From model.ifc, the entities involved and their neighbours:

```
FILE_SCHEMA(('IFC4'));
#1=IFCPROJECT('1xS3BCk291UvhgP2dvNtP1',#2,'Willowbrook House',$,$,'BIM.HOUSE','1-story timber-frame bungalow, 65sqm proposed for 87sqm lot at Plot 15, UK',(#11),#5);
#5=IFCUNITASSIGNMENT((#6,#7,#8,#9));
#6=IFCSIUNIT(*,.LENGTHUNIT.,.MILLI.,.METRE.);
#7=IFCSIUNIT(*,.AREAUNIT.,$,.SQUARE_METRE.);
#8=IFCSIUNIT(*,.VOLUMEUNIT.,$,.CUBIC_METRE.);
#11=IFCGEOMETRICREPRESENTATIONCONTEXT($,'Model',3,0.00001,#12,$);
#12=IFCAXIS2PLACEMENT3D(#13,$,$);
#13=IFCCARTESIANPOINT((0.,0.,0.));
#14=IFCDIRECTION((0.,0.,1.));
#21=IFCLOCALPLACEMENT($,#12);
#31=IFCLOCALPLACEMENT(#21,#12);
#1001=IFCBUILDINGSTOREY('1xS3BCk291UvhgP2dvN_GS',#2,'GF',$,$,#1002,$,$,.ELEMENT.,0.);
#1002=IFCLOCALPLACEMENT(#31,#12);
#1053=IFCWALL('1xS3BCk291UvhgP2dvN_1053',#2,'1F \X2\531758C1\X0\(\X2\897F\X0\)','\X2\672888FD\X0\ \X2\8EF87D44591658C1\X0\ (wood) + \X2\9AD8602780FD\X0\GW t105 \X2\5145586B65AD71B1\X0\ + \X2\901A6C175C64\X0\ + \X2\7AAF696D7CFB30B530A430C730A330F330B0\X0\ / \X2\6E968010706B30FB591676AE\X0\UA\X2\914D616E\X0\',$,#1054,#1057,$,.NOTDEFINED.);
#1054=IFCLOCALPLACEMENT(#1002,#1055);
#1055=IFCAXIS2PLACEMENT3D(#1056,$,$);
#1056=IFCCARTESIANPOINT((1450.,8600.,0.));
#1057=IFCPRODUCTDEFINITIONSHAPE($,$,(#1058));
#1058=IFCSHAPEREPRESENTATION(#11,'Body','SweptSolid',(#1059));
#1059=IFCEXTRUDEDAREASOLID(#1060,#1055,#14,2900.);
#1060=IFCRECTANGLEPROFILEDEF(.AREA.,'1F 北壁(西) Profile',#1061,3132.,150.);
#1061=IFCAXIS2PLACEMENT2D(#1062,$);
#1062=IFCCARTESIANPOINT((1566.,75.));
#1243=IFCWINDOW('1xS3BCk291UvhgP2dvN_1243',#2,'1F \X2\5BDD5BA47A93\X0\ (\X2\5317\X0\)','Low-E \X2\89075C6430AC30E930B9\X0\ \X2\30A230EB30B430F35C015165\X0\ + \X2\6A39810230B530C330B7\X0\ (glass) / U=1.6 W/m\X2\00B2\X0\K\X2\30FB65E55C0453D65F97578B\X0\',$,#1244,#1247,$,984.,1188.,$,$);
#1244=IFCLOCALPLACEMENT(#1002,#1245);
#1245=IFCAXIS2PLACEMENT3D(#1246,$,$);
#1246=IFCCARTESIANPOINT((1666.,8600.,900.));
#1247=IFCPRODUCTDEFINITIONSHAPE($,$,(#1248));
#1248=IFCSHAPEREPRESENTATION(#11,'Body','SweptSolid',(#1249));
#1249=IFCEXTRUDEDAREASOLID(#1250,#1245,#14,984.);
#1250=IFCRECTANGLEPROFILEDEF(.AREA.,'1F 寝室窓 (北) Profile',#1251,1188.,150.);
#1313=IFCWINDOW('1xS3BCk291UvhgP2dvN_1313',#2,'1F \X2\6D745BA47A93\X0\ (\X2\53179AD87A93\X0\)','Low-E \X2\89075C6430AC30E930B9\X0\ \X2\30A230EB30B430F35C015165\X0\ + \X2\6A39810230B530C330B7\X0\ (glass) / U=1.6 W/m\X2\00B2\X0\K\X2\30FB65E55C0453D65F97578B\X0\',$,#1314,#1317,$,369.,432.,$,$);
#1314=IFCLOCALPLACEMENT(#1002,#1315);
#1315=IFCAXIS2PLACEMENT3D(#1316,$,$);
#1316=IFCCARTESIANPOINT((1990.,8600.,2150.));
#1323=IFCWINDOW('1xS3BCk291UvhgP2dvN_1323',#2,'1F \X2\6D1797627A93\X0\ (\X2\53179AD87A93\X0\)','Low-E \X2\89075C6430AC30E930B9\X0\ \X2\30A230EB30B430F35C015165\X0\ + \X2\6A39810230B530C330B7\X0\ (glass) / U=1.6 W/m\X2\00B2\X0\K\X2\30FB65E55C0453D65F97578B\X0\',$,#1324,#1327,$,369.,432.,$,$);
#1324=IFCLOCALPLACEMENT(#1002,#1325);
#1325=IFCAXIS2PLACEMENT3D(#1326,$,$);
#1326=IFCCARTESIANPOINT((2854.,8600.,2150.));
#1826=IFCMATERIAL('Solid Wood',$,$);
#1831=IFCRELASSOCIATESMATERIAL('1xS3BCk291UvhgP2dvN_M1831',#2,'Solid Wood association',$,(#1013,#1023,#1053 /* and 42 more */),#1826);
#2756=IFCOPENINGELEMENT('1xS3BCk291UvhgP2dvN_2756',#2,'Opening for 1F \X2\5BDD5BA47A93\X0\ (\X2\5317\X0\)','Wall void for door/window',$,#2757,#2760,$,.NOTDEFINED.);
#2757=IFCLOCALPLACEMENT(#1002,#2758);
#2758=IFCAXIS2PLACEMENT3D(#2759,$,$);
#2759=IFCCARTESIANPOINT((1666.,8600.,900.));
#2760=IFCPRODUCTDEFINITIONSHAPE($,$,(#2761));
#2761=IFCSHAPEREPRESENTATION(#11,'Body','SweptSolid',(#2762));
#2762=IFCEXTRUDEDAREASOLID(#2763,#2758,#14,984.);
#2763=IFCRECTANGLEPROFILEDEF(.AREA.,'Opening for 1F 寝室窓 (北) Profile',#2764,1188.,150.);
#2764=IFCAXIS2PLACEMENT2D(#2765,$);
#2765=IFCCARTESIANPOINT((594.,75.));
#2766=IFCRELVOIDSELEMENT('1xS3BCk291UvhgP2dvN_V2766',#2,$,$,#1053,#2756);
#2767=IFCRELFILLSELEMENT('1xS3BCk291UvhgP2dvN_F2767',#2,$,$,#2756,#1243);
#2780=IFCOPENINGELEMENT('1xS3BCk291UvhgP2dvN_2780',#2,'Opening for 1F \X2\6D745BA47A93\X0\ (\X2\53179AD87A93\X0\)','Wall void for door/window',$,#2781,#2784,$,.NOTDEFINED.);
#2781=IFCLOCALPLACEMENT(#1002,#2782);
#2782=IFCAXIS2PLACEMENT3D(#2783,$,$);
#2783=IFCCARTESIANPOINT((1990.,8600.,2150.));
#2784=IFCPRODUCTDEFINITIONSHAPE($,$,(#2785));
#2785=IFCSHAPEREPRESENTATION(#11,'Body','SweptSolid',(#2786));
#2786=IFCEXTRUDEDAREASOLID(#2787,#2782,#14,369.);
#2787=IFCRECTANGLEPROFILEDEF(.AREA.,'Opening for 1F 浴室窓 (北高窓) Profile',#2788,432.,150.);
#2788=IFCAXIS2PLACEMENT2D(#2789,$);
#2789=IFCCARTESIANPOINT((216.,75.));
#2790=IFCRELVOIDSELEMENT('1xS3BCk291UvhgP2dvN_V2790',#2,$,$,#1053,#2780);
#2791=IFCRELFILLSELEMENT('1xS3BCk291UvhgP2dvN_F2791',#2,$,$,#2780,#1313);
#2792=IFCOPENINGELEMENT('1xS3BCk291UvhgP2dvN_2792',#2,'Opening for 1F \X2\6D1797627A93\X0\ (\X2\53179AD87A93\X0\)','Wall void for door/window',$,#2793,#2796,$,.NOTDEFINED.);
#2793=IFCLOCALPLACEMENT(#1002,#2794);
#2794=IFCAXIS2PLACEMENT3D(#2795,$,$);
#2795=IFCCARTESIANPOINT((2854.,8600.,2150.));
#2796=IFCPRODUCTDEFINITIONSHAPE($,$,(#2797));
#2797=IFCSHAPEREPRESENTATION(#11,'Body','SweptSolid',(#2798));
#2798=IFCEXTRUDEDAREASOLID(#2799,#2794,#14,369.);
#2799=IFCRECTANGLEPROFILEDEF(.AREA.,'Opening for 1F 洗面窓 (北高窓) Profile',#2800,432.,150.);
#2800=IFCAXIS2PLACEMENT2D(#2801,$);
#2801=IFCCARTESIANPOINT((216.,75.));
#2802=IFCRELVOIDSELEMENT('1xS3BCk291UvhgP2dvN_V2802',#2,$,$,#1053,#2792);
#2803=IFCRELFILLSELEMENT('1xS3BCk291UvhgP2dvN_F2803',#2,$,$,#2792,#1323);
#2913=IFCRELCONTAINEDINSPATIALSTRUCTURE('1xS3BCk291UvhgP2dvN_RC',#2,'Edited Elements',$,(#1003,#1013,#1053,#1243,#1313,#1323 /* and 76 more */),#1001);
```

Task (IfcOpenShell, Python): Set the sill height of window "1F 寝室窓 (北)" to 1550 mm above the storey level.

```python
import numpy as np
import ifcopenshell
import ifcopenshell.api.geometry
import ifcopenshell.geom
import ifcopenshell.util.element
import ifcopenshell.util.placement
import ifcopenshell.util.shape
import ifcopenshell.util.unit

model = ifcopenshell.open("model.ifc")
unit_scale = ifcopenshell.util.unit.calculate_unit_scale(model)

window = model.by_guid("1xS3BCk291UvhgP2dvN_1243")
opening = window.FillsVoids[0].RelatingOpeningElement
storey = ifcopenshell.util.element.get_container(window, ifc_class="IfcBuildingStorey")
level = ifcopenshell.util.placement.get_local_placement(storey.ObjectPlacement)[2, 3]

# The opening's origin need not be at the sill, so measure its lowest point.
shape = ifcopenshell.geom.create_shape(ifcopenshell.geom.settings(), opening)
bottom = ifcopenshell.util.shape.get_shape_bottom_elevation(shape, shape.geometry) / unit_scale
dz = level + 1550.0 - bottom

shift = np.array([0.0, 0.0, dz])
# The window is not placed relative to its opening, so move both.
for product in (opening, window):
    matrix = ifcopenshell.util.placement.get_local_placement(product.ObjectPlacement)
    matrix[:3, 3] += shift
    ifcopenshell.api.geometry.edit_object_placement(model, product=product, matrix=matrix, is_si=False)

print(f"moved by {dz * unit_scale:+.3f} m")

model.write("model_edited.ifc")
```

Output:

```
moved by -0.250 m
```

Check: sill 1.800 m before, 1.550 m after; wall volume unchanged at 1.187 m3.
